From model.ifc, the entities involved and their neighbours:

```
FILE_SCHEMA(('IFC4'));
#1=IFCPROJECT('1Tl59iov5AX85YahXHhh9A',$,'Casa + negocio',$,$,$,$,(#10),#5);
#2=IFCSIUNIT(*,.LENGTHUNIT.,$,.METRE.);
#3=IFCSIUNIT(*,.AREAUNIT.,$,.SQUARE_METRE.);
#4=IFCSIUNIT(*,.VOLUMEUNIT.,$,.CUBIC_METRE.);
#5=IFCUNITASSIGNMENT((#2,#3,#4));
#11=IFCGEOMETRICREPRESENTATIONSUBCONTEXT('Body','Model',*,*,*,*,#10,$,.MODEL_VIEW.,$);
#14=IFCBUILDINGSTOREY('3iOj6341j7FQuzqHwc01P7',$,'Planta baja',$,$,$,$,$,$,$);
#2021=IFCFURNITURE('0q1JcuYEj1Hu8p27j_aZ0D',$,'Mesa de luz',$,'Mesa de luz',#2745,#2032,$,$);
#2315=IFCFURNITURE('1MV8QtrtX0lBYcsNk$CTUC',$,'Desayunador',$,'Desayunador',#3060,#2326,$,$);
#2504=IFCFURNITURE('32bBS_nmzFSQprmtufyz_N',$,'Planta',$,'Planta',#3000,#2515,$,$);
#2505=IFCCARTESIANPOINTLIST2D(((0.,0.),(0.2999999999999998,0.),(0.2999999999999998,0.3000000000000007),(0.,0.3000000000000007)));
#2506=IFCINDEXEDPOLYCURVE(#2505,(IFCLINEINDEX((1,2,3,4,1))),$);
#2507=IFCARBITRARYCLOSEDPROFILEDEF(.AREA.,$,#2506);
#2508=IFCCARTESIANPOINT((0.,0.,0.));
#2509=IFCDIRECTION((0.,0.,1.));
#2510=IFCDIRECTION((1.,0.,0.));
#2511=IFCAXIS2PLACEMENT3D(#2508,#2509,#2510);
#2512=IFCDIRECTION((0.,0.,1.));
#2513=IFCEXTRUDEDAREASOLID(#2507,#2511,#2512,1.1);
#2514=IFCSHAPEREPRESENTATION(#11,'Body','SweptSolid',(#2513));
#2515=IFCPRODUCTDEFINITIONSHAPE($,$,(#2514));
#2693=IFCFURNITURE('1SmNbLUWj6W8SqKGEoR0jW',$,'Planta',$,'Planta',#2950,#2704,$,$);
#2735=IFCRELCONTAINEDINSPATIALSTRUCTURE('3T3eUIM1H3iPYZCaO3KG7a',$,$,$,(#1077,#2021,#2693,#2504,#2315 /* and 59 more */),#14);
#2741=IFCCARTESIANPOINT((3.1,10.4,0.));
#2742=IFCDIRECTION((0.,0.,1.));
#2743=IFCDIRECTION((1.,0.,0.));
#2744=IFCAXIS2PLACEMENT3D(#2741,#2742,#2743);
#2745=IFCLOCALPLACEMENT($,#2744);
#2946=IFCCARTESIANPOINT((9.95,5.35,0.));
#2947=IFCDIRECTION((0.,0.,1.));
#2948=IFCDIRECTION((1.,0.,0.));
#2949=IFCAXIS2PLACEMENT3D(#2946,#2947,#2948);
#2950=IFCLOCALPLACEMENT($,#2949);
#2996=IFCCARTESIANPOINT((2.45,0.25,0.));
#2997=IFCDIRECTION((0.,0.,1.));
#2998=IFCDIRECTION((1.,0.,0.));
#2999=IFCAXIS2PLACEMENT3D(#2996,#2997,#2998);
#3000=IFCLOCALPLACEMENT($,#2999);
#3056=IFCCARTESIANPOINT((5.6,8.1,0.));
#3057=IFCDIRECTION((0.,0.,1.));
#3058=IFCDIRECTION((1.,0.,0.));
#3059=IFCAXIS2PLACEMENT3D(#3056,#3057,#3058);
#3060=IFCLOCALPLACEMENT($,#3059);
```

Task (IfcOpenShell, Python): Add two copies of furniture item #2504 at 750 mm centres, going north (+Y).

```python
import numpy as np
import ifcopenshell
import ifcopenshell.api.geometry
import ifcopenshell.api.root
import ifcopenshell.util.element
import ifcopenshell.util.placement

model = ifcopenshell.open("model.ifc")

source = model.by_guid("32bBS_nmzFSQprmtufyz_N")
base = ifcopenshell.util.placement.get_local_placement(source.ObjectPlacement)
step = np.array([0.0, 1.0, 0.0]) * 0.75

for i in range(1, 3):
    copy = ifcopenshell.api.root.copy_class(model, product=source)
    copy.Representation = ifcopenshell.util.element.copy_deep(
        model, source.Representation, exclude=["IfcGeometricRepresentationContext", "IfcRepresentationMap"]
    )
    matrix = base.copy()
    matrix[:3, 3] += i * step
    print("added at", matrix[:3, 3].round(3) + 0.0)
    ifcopenshell.api.geometry.edit_object_placement(model, product=copy, matrix=matrix, is_si=False)

model.write("model_rev.ifc")
```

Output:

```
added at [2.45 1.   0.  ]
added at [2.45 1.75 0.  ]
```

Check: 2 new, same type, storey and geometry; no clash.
